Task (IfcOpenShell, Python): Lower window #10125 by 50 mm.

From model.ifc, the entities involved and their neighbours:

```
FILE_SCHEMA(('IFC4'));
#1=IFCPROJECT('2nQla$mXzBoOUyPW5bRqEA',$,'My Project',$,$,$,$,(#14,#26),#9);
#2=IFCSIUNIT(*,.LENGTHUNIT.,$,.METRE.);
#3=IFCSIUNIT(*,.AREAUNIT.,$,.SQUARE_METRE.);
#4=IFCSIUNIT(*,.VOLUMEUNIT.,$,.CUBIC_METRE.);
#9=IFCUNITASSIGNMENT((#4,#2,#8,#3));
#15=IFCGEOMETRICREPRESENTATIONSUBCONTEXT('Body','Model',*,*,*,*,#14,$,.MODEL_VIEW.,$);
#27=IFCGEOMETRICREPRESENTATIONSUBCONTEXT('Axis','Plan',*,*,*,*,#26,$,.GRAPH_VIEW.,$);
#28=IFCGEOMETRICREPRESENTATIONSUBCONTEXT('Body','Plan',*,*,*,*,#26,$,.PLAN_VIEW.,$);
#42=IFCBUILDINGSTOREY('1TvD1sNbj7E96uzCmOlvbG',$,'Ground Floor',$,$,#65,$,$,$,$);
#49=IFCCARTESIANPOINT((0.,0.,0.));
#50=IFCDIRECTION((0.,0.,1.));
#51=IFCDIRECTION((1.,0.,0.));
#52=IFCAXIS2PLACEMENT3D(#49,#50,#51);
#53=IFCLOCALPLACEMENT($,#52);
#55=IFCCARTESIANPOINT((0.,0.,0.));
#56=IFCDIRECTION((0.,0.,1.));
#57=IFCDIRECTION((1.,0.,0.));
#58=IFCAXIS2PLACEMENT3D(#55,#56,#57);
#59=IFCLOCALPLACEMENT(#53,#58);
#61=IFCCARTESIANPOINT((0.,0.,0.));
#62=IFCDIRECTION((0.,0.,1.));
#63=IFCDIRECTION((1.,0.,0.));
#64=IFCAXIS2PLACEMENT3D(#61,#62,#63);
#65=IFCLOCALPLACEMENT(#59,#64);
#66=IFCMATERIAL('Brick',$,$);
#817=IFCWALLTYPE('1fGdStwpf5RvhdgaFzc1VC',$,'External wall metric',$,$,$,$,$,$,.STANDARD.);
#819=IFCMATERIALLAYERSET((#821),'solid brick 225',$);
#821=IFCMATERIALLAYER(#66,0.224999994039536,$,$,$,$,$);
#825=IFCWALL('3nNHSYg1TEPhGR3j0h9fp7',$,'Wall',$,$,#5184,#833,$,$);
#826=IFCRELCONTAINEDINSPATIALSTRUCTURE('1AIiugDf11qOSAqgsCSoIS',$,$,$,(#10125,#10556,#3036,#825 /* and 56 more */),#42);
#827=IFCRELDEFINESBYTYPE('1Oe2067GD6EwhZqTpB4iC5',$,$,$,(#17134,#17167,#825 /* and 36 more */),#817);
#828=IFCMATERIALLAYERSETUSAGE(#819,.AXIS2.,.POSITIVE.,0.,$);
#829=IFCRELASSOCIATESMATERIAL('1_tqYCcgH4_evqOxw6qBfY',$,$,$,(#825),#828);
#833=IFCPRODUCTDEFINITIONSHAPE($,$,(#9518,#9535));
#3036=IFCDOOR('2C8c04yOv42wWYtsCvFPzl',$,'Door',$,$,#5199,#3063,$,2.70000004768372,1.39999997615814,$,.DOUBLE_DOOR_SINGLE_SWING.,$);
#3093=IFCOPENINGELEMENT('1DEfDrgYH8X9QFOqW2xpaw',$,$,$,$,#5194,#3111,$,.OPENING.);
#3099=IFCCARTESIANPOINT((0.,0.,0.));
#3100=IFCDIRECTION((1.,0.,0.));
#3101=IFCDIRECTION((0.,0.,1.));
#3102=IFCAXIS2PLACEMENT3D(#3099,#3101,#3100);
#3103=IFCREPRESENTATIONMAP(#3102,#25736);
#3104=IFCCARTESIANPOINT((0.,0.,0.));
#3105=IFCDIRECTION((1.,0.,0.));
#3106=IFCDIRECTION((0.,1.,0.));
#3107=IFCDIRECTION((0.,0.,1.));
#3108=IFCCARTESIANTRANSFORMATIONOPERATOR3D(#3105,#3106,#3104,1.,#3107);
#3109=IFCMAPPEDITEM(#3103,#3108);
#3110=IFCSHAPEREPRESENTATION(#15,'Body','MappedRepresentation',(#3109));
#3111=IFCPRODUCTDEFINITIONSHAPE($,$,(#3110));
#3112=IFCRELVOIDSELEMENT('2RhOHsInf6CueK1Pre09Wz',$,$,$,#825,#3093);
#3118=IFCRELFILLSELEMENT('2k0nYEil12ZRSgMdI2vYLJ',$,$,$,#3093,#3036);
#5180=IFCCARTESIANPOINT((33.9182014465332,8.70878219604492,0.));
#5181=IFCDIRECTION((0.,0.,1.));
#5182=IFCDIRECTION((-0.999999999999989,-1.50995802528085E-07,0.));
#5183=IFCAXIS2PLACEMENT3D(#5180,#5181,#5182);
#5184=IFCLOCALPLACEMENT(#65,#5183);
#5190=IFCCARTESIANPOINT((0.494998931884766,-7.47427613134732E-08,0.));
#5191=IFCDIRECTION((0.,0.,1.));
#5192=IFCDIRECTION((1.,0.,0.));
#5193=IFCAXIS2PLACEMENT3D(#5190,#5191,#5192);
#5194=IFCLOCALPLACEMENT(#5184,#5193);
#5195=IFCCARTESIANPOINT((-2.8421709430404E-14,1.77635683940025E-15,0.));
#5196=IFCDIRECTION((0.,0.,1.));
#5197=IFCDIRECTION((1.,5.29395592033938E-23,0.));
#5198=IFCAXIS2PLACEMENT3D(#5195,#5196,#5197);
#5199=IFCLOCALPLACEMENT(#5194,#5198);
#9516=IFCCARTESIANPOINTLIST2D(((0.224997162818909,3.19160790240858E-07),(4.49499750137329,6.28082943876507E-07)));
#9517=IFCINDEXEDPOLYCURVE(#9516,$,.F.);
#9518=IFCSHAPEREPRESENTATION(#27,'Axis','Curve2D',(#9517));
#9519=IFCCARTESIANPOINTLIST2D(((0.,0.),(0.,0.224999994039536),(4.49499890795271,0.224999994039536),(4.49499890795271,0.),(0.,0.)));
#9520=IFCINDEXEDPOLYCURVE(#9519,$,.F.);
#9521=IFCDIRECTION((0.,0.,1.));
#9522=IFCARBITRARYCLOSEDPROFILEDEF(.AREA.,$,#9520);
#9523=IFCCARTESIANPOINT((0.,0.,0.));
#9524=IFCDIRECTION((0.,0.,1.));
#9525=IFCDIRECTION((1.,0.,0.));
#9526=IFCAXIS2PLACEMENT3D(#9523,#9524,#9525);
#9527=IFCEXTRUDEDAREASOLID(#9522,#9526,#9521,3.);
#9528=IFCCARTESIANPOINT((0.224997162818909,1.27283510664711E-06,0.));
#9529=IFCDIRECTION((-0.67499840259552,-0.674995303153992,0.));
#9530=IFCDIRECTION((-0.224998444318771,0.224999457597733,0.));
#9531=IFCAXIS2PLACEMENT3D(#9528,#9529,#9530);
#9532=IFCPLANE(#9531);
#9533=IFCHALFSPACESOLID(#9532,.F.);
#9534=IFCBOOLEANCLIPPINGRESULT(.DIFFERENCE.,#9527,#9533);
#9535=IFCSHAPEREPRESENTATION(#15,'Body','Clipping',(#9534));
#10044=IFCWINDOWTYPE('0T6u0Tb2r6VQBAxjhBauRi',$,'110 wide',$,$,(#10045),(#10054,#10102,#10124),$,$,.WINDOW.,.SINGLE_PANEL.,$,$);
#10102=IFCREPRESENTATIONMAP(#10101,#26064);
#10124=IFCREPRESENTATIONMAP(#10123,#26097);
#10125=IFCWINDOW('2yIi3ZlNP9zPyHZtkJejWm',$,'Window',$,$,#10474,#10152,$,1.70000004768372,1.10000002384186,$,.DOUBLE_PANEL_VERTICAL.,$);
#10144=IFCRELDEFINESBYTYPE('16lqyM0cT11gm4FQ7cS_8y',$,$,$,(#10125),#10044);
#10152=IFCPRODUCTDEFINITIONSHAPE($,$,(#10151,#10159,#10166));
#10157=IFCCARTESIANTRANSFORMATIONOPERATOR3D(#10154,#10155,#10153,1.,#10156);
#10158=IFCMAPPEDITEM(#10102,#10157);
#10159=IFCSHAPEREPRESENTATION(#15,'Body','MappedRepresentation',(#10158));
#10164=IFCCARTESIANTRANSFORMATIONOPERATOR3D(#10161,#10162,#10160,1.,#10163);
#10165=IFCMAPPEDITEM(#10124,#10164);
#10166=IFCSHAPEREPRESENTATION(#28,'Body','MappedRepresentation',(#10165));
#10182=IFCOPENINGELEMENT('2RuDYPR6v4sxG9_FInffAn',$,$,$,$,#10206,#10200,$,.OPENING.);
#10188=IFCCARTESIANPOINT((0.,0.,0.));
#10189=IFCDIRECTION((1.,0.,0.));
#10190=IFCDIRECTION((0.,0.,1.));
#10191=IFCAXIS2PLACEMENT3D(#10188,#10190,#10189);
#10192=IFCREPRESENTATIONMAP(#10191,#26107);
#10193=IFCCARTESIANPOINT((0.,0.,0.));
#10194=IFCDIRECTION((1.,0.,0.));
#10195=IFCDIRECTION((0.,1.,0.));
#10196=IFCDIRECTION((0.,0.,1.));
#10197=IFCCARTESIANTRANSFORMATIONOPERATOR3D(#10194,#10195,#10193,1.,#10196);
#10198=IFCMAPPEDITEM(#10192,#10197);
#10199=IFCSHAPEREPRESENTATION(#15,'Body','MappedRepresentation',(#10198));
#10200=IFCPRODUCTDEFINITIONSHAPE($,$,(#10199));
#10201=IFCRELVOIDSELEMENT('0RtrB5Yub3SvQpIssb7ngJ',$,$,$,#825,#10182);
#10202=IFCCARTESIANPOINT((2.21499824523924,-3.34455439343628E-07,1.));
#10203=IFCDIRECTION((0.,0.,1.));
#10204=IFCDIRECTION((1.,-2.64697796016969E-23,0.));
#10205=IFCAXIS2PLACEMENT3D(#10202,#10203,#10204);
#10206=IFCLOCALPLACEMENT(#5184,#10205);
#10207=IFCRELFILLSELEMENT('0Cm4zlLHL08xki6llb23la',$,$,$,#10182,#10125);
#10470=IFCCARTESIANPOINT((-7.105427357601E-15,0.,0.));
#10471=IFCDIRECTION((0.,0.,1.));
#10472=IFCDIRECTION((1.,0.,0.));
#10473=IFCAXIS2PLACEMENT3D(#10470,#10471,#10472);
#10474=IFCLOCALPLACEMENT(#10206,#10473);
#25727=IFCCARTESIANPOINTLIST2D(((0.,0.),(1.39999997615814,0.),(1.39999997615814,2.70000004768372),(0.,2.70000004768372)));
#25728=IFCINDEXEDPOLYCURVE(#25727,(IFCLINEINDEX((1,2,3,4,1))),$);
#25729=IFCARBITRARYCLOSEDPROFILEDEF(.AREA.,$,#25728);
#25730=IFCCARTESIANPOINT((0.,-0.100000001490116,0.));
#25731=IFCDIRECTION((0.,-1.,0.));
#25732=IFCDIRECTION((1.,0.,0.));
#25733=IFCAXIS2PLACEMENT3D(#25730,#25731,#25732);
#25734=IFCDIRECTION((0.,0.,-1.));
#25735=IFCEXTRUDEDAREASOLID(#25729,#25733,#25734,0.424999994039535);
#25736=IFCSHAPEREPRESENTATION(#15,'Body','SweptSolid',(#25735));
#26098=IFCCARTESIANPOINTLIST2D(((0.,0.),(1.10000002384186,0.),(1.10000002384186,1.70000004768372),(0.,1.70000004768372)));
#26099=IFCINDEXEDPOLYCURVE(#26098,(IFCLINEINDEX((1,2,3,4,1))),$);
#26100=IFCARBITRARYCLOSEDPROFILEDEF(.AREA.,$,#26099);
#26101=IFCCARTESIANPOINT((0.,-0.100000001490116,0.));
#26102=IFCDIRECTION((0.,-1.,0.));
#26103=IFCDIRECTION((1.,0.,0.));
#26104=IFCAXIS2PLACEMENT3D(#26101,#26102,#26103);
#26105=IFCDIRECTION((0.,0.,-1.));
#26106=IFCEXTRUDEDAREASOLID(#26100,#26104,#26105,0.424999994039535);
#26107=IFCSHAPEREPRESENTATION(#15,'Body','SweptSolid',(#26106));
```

```python
import numpy as np
import ifcopenshell
import ifcopenshell.api.geometry
import ifcopenshell.util.placement
import ifcopenshell.util.unit

model = ifcopenshell.open("model.ifc")
unit_scale = ifcopenshell.util.unit.calculate_unit_scale(model)

window = model.by_guid("2yIi3ZlNP9zPyHZtkJejWm")
opening = window.FillsVoids[0].RelatingOpeningElement
dz = -0.05

shift = np.array([0.0, 0.0, dz])
# The window is placed relative to its opening, so it follows when the opening moves.
matrix = ifcopenshell.util.placement.get_local_placement(opening.ObjectPlacement)
matrix[:3, 3] += shift
ifcopenshell.api.geometry.edit_object_placement(
    model, product=opening, matrix=matrix, is_si=False, should_transform_children=True
)

print(f"moved by {dz * unit_scale:+.3f} m")

model.write("model_rev.ifc")
```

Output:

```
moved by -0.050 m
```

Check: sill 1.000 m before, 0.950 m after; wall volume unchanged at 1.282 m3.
